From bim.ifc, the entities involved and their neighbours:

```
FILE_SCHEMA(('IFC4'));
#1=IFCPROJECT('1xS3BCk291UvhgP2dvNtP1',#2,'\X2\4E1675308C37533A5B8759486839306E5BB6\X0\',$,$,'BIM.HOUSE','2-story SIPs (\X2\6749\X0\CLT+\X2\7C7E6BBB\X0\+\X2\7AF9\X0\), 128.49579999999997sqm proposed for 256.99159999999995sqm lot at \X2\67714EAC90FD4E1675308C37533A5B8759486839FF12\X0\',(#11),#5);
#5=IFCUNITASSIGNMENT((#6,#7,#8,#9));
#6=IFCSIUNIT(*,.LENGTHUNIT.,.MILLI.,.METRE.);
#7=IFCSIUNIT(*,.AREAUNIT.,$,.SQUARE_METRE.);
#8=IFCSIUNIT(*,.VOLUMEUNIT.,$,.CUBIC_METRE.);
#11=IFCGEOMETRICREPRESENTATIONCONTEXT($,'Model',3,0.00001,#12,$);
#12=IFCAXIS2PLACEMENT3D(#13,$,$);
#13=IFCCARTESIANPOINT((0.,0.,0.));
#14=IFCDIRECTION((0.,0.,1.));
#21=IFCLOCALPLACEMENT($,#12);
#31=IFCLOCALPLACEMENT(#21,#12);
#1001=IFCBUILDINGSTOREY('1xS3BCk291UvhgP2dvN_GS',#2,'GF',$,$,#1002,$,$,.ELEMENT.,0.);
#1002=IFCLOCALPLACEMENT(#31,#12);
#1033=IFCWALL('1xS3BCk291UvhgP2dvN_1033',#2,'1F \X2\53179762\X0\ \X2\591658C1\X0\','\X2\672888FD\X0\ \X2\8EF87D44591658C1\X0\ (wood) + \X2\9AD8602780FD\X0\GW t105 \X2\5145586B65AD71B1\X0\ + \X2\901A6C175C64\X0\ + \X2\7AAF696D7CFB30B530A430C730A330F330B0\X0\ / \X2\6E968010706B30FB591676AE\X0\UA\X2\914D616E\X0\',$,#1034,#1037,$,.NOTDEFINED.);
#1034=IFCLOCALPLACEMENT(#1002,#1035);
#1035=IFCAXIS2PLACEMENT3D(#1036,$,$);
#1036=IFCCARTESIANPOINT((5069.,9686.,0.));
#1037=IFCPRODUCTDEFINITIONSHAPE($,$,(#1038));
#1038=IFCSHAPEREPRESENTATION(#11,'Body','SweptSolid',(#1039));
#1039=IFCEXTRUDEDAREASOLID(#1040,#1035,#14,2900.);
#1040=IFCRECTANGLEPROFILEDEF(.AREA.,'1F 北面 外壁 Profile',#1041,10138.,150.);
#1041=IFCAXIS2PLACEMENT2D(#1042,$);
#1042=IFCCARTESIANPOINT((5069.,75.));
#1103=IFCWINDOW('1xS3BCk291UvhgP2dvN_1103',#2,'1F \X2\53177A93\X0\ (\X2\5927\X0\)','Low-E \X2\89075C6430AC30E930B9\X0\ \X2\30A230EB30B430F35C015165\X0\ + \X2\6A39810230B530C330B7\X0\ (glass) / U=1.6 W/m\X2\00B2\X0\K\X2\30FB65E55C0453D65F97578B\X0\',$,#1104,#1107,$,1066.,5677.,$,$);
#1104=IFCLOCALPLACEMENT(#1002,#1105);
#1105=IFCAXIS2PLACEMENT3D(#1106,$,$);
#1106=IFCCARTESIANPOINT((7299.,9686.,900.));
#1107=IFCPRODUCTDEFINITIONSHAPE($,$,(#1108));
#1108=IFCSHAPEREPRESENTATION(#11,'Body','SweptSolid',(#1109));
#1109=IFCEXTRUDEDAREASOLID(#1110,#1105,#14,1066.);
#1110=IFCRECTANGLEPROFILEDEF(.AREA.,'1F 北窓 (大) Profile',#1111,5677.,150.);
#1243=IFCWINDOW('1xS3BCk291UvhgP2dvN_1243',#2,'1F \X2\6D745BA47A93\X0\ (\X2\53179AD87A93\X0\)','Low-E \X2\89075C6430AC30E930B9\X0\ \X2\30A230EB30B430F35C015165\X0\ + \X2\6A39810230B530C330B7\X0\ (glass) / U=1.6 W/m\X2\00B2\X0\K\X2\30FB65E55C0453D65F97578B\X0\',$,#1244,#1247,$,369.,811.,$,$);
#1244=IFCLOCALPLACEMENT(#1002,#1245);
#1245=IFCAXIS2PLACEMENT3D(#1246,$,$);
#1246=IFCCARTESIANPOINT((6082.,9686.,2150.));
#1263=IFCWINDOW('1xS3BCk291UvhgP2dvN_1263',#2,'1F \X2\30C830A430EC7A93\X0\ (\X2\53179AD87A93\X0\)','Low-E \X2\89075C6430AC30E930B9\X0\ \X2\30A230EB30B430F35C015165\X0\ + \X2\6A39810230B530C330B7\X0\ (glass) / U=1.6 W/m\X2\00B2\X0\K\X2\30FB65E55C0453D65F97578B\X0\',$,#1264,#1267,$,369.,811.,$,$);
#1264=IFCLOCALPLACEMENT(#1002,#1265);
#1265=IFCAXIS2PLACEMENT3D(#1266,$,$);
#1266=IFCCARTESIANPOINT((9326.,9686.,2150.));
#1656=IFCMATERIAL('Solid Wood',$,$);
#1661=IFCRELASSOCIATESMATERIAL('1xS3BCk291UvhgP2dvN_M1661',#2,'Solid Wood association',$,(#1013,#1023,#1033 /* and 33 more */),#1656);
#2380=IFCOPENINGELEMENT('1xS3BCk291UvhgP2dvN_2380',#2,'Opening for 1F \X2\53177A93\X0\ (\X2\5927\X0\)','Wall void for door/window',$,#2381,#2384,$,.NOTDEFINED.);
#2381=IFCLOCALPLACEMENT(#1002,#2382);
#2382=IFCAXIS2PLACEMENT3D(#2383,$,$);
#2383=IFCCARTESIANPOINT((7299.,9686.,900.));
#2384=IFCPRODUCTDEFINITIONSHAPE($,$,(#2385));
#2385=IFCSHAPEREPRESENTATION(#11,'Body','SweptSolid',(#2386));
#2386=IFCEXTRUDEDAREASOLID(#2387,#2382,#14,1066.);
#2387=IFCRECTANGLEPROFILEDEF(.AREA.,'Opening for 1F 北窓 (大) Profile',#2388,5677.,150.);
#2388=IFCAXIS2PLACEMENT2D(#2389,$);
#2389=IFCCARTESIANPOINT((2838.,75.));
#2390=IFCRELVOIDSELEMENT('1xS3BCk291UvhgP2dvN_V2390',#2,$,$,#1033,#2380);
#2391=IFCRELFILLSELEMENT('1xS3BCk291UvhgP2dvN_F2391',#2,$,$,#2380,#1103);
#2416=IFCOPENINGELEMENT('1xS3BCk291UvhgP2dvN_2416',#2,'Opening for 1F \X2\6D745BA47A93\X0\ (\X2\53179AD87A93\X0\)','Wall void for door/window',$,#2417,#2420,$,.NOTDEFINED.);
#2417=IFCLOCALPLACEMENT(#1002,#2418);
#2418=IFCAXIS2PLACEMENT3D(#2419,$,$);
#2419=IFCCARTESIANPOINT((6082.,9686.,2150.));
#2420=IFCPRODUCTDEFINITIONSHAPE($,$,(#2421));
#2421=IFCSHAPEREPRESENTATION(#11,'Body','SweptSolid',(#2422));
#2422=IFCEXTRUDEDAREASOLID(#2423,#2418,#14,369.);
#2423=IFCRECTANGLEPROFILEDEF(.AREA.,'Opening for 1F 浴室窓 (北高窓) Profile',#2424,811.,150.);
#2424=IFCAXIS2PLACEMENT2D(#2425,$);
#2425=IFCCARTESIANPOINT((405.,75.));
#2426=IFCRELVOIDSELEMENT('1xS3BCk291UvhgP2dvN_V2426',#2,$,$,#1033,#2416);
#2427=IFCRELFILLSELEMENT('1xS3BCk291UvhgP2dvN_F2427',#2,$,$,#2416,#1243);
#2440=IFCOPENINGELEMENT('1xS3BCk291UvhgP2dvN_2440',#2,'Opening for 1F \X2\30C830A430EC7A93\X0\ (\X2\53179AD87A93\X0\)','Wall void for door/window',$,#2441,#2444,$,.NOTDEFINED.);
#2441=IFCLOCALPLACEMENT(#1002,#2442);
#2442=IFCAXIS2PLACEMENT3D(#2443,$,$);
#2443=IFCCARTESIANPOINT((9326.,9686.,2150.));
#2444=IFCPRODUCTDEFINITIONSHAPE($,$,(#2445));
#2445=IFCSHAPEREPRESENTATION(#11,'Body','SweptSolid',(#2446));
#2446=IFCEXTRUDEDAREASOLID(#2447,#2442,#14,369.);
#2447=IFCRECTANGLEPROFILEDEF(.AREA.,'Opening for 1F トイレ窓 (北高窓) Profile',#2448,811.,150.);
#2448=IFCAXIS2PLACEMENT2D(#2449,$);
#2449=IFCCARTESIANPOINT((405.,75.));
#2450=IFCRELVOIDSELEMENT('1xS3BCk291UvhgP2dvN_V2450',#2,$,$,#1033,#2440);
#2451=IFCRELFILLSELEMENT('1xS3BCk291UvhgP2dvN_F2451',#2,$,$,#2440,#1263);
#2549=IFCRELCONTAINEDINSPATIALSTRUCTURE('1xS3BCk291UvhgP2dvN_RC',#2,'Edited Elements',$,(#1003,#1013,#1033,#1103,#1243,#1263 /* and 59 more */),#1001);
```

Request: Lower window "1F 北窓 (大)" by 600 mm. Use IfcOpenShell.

```python
import numpy as np
import ifcopenshell
import ifcopenshell.api.geometry
import ifcopenshell.util.placement
import ifcopenshell.util.unit

model = ifcopenshell.open("bim.ifc")
unit_scale = ifcopenshell.util.unit.calculate_unit_scale(model)

window = model.by_guid("1xS3BCk291UvhgP2dvN_1103")
opening = window.FillsVoids[0].RelatingOpeningElement
dz = -0.6 / unit_scale

shift = np.array([0.0, 0.0, dz])
# The window is not placed relative to its opening, so move both.
for product in (opening, window):
    matrix = ifcopenshell.util.placement.get_local_placement(product.ObjectPlacement)
    matrix[:3, 3] += shift
    ifcopenshell.api.geometry.edit_object_placement(model, product=product, matrix=matrix, is_si=False)

print(f"moved by {dz * unit_scale:+.3f} m")

model.write("bim_rev.ifc")
```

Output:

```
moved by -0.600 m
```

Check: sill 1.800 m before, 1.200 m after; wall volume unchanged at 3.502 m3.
